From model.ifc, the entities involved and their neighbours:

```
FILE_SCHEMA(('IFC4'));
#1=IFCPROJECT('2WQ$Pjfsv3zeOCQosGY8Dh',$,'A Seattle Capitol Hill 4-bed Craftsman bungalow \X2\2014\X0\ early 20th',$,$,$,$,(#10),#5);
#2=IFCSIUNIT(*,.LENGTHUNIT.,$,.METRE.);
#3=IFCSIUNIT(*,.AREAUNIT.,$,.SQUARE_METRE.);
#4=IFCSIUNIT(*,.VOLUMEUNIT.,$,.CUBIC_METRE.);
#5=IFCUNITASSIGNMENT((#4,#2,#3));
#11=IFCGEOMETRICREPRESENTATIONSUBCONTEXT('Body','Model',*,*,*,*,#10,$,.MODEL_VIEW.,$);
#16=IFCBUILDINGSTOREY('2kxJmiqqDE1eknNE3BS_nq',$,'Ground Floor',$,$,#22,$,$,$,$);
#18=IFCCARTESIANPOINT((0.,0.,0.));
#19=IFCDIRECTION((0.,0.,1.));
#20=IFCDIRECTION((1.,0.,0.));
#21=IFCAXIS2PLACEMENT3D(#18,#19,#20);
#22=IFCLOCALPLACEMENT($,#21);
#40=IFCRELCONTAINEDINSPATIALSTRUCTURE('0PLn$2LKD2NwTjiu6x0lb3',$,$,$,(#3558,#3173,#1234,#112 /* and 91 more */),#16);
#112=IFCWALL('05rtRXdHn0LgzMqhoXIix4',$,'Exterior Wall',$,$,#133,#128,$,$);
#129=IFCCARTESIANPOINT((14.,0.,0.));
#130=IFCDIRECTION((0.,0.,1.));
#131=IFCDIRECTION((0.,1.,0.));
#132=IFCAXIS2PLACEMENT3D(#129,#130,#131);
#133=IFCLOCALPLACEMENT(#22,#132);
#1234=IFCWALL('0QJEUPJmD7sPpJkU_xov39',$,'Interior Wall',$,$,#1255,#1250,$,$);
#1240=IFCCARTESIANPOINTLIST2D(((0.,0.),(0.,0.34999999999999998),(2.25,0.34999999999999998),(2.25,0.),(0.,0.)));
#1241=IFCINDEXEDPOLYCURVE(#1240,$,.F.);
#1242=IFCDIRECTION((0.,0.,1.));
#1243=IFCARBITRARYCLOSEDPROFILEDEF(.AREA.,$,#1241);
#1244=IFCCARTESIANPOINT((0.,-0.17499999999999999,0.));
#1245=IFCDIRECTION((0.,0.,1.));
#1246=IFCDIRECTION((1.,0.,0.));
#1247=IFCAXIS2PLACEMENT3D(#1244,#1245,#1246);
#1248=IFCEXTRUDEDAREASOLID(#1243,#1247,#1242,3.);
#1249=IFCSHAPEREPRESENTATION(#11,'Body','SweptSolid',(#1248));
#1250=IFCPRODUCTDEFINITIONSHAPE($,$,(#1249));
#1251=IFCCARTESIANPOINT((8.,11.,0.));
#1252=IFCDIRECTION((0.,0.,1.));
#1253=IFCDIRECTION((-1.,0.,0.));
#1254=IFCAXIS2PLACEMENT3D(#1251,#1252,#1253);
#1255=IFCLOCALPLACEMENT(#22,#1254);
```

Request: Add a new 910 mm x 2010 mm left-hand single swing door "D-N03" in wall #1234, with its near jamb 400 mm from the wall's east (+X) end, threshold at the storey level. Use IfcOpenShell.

```python
import numpy as np
import ifcopenshell
import ifcopenshell.api.feature
import ifcopenshell.api.geometry
import ifcopenshell.api.root
import ifcopenshell.api.spatial
import ifcopenshell.geom
import ifcopenshell.util.element
import ifcopenshell.util.placement
import ifcopenshell.util.representation
import ifcopenshell.util.shape
import ifcopenshell.util.unit

model = ifcopenshell.open("model.ifc")
unit_scale = ifcopenshell.util.unit.calculate_unit_scale(model)
settings = ifcopenshell.geom.settings()


def volume(element):
    """Net volume in cubic metres, openings subtracted."""
    shape = ifcopenshell.geom.create_shape(settings, element)
    return ifcopenshell.util.shape.get_volume(shape.geometry)


wall = model.by_guid("0QJEUPJmD7sPpJkU_xov39")
storey = ifcopenshell.util.element.get_container(wall, ifc_class="IfcBuildingStorey")
context = ifcopenshell.util.representation.get_context(model, "Model", "Body", "MODEL_VIEW")
before = volume(wall)

width, height, from_end, sill = 0.91, 2.01, 0.4, 0.0  # metres

# The wall runs along its own X axis, and the end named is its -X end.
wall_shape = ifcopenshell.geom.create_shape(settings, wall)
x, y, z = ifcopenshell.util.shape.get_vertices(wall_shape.geometry).T
start = x.min() + from_end
face, thickness = float(y.min()), float(y.max() - y.min())
wall_matrix = ifcopenshell.util.placement.get_local_placement(wall.ObjectPlacement)
level = ifcopenshell.util.placement.get_local_placement(storey.ObjectPlacement)[2, 3]


def in_wall(x, y):
    """Placement at x, y metres in the wall's axes, at sill height."""
    matrix = wall_matrix.copy()
    matrix[:, 3] = wall_matrix @ np.array([x / unit_scale, y / unit_scale, 0.0, 1.0])
    matrix[2, 3] = level + sill / unit_scale
    return matrix


# Opening: a box that overshoots both wall faces by 50 mm.
opening = ifcopenshell.api.root.create_entity(model, ifc_class="IfcOpeningElement", predefined_type="OPENING")
box = ifcopenshell.api.geometry.add_wall_representation(
    model, context=context, length=width, height=height, thickness=thickness + 0.1
)
ifcopenshell.api.geometry.assign_representation(model, product=opening, representation=box)
ifcopenshell.api.geometry.edit_object_placement(model, product=opening, matrix=in_wall(start, face - 0.05), is_si=False)
ifcopenshell.api.feature.add_feature(model, feature=opening, element=wall)

door = ifcopenshell.api.root.create_entity(model, ifc_class="IfcDoor", name="D-N03", predefined_type="DOOR")
door.OverallWidth, door.OverallHeight = width / unit_scale, height / unit_scale
door.OperationType = "SINGLE_SWING_LEFT"
body = ifcopenshell.api.geometry.add_door_representation(
    model,
    context=context,
    overall_width=door.OverallWidth,
    overall_height=door.OverallHeight,
    operation_type="SINGLE_SWING_LEFT",
    lining_properties={"LiningDepth": thickness / unit_scale, "ThresholdDepth": thickness / unit_scale},
)
ifcopenshell.api.geometry.assign_representation(model, product=door, representation=body)
ifcopenshell.api.spatial.assign_container(model, products=[door], relating_structure=storey)
ifcopenshell.api.feature.add_filling(model, opening=opening, element=door)

# The lining spans the wall, so the door starts at the wall face.
ifcopenshell.api.geometry.edit_object_placement(model, product=door, matrix=in_wall(start, face), is_si=False)

after = volume(wall)

print(f"wall volume {before:.3f} -> {after:.3f} m3")

model.write("model_updated.ifc")
```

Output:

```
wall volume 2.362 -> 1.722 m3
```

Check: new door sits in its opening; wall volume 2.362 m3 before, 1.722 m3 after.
